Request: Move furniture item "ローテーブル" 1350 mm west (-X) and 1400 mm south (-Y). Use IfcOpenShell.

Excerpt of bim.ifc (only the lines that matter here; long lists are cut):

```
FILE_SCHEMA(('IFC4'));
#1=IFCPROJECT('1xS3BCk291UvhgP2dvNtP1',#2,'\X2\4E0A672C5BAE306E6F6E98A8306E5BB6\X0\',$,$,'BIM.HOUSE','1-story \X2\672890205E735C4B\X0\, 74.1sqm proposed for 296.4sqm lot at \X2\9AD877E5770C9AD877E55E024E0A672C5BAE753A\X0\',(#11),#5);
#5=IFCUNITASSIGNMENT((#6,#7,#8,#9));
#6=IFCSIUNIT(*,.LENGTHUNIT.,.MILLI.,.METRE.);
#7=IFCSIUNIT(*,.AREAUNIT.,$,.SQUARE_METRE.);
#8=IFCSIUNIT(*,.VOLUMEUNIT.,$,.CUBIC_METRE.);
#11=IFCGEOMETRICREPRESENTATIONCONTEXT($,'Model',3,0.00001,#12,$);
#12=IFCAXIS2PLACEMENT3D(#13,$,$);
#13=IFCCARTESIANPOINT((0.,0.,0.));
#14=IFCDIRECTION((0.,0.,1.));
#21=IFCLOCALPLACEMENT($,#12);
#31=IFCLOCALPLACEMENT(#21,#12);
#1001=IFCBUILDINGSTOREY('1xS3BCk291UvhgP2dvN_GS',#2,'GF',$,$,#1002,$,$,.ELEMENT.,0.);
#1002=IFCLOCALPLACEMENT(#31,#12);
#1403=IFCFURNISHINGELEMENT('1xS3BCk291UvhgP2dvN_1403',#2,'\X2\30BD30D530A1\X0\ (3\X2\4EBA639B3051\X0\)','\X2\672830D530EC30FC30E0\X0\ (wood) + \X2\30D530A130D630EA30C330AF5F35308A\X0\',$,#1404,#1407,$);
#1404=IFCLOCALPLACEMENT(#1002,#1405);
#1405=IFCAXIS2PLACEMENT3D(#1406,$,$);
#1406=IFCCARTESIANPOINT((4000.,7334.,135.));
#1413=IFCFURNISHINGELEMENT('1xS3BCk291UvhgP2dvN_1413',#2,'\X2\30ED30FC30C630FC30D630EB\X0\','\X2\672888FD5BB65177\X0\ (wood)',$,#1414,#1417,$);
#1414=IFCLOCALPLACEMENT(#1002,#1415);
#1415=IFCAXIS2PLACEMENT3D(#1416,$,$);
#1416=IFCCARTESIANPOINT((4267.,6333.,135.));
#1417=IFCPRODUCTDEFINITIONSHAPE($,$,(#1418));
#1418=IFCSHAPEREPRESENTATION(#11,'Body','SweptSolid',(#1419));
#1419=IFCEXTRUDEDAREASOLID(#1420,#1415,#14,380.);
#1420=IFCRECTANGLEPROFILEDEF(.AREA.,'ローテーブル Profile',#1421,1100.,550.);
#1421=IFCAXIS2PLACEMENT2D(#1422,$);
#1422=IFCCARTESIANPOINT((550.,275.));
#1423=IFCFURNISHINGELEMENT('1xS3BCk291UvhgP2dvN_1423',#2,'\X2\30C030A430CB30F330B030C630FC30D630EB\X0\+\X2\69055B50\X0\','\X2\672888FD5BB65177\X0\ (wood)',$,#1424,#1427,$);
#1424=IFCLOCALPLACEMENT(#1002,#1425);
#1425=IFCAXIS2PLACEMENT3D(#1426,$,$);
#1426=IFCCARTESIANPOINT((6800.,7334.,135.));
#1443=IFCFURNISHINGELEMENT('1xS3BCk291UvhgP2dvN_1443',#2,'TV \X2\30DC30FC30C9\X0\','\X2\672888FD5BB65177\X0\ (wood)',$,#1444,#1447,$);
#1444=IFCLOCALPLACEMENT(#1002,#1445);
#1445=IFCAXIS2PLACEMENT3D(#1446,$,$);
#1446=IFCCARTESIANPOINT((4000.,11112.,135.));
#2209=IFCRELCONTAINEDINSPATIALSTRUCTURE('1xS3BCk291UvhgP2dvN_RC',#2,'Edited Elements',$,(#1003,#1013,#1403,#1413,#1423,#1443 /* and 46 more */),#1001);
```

```python
import ifcopenshell
import ifcopenshell.api.geometry
import ifcopenshell.util.placement

model = ifcopenshell.open("bim.ifc")

item = model.by_guid("1xS3BCk291UvhgP2dvN_1413")
matrix = ifcopenshell.util.placement.get_local_placement(item.ObjectPlacement)
matrix[0, 3] -= 1350.0
matrix[1, 3] -= 1400.0
ifcopenshell.api.geometry.edit_object_placement(model, product=item, matrix=matrix, is_si=False)

print(ifcopenshell.util.placement.get_local_placement(item.ObjectPlacement).round(3) + 0.0)

model.write("bim_rev.ifc")
```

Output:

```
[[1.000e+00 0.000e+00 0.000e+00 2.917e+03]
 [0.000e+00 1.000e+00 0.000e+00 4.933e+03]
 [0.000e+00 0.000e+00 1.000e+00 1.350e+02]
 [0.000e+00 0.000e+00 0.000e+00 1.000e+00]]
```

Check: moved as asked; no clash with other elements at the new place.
